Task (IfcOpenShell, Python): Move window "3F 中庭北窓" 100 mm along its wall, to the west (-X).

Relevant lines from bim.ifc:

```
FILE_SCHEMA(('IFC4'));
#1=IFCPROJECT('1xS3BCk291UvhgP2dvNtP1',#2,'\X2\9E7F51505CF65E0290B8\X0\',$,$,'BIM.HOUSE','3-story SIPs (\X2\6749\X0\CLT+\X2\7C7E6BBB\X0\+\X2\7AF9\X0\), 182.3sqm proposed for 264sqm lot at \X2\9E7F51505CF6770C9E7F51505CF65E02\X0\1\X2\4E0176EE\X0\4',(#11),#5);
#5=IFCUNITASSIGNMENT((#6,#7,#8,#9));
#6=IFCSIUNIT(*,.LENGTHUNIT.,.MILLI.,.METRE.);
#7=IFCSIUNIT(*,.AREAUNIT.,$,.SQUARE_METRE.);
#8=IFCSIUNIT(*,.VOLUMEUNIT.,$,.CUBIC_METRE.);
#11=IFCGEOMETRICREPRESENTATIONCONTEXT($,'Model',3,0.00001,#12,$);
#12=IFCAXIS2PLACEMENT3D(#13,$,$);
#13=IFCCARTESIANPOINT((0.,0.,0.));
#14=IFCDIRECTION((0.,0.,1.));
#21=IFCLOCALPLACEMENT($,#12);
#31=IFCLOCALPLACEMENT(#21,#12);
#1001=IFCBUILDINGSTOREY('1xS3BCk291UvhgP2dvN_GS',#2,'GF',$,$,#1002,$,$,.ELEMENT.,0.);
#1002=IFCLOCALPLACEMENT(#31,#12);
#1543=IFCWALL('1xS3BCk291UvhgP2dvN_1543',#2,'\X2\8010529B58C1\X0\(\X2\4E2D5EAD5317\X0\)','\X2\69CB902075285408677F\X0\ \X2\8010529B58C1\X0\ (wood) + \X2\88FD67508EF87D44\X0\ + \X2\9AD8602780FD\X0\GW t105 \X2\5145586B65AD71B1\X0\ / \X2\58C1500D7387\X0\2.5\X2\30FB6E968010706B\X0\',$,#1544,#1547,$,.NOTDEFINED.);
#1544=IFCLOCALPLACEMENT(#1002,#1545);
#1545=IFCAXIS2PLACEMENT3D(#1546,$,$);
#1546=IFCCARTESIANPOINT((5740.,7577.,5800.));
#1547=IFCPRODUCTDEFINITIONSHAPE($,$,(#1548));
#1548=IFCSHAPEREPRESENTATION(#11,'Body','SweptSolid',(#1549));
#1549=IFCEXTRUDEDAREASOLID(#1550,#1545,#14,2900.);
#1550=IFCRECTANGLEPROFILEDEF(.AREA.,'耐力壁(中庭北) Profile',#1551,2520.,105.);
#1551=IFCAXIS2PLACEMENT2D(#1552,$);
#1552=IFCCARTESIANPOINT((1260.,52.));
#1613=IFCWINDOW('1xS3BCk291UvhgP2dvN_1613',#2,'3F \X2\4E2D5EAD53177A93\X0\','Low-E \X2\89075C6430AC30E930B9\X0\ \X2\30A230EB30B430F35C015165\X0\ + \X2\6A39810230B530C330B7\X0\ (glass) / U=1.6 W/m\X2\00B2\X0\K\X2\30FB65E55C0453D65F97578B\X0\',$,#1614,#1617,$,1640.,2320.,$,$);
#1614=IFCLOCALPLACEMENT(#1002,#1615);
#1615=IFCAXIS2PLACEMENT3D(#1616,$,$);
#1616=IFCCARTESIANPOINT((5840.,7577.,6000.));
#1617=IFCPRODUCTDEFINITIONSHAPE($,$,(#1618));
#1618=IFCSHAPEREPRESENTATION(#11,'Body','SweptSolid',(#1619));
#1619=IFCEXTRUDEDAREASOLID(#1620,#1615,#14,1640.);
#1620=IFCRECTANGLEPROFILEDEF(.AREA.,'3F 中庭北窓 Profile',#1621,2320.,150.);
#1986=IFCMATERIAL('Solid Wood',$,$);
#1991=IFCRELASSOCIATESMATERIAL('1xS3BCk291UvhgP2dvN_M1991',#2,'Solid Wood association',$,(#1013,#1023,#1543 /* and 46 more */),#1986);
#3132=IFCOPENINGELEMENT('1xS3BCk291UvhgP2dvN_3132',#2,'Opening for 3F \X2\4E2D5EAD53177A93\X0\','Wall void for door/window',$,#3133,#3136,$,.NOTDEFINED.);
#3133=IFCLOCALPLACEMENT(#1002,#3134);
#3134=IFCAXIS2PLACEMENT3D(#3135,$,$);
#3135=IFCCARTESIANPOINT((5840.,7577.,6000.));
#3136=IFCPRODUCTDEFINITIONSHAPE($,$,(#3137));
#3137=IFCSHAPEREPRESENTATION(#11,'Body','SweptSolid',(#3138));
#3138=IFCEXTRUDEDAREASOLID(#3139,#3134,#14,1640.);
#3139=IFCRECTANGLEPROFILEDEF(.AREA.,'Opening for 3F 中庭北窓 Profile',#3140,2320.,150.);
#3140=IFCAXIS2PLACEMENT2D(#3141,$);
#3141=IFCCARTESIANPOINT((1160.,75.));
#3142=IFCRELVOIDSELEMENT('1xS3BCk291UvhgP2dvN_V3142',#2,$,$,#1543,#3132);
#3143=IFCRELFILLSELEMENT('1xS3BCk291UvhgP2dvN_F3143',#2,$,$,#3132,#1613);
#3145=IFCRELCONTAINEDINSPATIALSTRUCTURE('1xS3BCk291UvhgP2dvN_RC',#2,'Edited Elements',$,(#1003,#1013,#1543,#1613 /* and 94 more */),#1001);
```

```python
import ifcopenshell
import ifcopenshell.api.geometry
import ifcopenshell.util.placement

model = ifcopenshell.open("bim.ifc")

window = model.by_guid("1xS3BCk291UvhgP2dvN_1613")
opening = window.FillsVoids[0].RelatingOpeningElement
wall = opening.VoidsElements[0].RelatingBuildingElement

wall_matrix = ifcopenshell.util.placement.get_local_placement(wall.ObjectPlacement)
shift = wall_matrix[:3, 0] * -100.0
before = ifcopenshell.util.placement.get_local_placement(window.ObjectPlacement)[:3, 3].copy()

# The window is not placed relative to its opening, so move both.
for product in (opening, window):
    matrix = ifcopenshell.util.placement.get_local_placement(product.ObjectPlacement)
    matrix[:3, 3] += shift
    ifcopenshell.api.geometry.edit_object_placement(model, product=product, matrix=matrix, is_si=False)

after = ifcopenshell.util.placement.get_local_placement(window.ObjectPlacement)[:3, 3]
print("window moved by", (after - before).round(3) + 0.0)

model.write("bim_edited.ifc")
```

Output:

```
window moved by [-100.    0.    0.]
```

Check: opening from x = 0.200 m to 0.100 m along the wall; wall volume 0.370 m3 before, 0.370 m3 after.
